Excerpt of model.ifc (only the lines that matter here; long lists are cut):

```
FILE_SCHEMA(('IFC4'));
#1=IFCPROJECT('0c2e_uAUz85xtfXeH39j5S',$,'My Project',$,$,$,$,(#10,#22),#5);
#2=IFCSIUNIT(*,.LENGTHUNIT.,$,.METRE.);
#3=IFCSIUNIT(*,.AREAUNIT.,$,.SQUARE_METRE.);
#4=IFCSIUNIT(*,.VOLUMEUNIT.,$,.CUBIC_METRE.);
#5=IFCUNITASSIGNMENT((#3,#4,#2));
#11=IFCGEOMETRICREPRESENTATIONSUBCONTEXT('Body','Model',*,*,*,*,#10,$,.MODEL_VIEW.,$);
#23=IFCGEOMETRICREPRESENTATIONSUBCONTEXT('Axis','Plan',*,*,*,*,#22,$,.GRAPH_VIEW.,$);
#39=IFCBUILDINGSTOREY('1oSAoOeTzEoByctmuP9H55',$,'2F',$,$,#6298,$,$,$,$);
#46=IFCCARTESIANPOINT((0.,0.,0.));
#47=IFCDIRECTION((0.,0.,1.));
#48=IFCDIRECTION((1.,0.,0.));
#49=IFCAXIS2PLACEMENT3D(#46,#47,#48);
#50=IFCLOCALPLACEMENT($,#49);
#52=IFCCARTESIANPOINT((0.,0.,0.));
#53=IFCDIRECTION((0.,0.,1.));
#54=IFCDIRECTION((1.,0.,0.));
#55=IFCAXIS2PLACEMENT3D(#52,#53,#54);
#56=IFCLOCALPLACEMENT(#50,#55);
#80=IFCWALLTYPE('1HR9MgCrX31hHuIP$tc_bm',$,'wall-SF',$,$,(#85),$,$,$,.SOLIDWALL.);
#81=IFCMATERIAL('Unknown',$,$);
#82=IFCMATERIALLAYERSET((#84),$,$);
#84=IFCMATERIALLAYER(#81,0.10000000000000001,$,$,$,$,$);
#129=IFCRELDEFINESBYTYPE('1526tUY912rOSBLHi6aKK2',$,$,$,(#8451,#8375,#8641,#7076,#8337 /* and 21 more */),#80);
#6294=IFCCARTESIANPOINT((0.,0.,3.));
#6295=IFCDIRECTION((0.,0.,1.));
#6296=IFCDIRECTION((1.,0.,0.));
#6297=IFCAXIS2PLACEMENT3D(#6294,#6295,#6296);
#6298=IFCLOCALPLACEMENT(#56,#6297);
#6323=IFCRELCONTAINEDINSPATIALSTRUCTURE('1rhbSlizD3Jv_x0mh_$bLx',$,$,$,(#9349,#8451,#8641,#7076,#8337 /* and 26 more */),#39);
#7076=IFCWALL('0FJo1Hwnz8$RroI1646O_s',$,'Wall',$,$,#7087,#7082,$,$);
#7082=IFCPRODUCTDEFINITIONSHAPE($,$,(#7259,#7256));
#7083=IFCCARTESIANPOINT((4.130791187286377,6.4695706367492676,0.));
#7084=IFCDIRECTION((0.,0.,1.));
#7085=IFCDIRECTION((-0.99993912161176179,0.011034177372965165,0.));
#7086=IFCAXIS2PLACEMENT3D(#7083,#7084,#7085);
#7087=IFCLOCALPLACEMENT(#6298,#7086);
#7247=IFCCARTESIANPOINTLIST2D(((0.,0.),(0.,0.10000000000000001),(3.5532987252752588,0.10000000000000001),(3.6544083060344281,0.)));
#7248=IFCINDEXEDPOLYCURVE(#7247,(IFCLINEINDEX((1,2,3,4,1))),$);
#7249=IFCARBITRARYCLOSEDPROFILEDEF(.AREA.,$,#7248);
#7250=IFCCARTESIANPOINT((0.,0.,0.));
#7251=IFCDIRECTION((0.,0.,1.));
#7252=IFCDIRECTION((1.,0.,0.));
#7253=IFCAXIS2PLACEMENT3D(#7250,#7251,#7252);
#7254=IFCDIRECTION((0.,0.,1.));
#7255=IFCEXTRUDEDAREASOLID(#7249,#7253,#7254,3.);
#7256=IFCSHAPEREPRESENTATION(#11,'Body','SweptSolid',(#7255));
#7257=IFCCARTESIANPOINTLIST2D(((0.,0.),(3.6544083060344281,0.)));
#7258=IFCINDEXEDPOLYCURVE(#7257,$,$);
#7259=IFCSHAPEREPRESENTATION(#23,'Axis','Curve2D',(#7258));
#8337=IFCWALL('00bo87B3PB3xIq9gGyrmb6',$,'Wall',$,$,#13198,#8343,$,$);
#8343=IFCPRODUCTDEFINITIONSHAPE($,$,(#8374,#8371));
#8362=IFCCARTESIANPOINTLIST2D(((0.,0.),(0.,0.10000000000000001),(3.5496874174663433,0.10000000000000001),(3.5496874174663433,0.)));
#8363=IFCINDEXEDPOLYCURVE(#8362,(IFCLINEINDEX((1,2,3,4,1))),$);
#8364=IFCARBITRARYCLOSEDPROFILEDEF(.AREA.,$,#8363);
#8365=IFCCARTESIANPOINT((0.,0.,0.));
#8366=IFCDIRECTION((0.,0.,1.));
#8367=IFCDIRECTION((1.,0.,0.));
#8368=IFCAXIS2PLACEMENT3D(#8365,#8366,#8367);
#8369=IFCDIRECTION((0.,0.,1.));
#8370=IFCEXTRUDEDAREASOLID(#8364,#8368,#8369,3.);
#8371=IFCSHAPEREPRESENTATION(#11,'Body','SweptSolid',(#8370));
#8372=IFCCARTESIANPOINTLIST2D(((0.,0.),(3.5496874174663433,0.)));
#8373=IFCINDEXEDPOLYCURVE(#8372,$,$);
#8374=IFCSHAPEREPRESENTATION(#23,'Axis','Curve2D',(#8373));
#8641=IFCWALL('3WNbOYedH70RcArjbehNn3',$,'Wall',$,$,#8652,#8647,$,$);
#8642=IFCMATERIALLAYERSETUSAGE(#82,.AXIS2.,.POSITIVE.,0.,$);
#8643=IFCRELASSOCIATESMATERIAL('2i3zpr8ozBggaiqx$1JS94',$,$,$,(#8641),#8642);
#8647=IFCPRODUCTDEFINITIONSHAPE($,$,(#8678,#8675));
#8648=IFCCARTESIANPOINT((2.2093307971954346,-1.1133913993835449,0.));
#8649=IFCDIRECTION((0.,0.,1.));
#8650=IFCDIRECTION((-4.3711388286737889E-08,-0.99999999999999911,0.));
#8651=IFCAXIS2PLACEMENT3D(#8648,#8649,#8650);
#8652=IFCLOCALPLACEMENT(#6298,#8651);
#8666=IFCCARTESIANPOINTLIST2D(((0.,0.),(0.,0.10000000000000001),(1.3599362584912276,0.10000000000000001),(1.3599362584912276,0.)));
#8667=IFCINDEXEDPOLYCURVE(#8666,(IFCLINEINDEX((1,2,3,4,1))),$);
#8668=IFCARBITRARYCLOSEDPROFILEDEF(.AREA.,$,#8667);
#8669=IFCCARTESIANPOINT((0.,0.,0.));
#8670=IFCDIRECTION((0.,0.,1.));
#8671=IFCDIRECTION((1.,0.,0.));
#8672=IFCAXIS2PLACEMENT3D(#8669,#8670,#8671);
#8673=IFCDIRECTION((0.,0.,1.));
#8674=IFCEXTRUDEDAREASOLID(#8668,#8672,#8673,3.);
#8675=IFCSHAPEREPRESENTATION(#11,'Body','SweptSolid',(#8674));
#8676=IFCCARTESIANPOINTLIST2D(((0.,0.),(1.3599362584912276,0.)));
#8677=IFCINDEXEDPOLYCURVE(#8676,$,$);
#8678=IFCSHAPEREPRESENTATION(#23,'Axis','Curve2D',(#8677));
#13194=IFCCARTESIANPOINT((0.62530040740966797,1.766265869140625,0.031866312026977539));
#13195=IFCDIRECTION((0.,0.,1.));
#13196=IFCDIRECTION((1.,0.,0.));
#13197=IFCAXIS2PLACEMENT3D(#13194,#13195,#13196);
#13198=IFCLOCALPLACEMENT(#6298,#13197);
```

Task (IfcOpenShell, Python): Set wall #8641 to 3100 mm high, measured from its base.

```python
import ifcopenshell
import ifcopenshell.geom
import ifcopenshell.util.representation
import ifcopenshell.util.shape
import ifcopenshell.util.unit

model = ifcopenshell.open("model.ifc")
unit_scale = ifcopenshell.util.unit.calculate_unit_scale(model)
settings = ifcopenshell.geom.settings()


def volume(element):
    """Net volume in cubic metres, openings subtracted."""
    shape = ifcopenshell.geom.create_shape(settings, element)
    return ifcopenshell.util.shape.get_volume(shape.geometry)


wall = model.by_id(8641)
before = volume(wall)

body = ifcopenshell.util.representation.get_representation(wall, "Model", "Body")
solid = body.Items[0]
old_height = solid.Depth
solid.Depth = 3.1 / unit_scale
after = volume(wall)

print(f"height {old_height:g} -> {solid.Depth:g}, volume {before:.3f} -> {after:.3f} m3")

model.write("model_v2.ifc")
```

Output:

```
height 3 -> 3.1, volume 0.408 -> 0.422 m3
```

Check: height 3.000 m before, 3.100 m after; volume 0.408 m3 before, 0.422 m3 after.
